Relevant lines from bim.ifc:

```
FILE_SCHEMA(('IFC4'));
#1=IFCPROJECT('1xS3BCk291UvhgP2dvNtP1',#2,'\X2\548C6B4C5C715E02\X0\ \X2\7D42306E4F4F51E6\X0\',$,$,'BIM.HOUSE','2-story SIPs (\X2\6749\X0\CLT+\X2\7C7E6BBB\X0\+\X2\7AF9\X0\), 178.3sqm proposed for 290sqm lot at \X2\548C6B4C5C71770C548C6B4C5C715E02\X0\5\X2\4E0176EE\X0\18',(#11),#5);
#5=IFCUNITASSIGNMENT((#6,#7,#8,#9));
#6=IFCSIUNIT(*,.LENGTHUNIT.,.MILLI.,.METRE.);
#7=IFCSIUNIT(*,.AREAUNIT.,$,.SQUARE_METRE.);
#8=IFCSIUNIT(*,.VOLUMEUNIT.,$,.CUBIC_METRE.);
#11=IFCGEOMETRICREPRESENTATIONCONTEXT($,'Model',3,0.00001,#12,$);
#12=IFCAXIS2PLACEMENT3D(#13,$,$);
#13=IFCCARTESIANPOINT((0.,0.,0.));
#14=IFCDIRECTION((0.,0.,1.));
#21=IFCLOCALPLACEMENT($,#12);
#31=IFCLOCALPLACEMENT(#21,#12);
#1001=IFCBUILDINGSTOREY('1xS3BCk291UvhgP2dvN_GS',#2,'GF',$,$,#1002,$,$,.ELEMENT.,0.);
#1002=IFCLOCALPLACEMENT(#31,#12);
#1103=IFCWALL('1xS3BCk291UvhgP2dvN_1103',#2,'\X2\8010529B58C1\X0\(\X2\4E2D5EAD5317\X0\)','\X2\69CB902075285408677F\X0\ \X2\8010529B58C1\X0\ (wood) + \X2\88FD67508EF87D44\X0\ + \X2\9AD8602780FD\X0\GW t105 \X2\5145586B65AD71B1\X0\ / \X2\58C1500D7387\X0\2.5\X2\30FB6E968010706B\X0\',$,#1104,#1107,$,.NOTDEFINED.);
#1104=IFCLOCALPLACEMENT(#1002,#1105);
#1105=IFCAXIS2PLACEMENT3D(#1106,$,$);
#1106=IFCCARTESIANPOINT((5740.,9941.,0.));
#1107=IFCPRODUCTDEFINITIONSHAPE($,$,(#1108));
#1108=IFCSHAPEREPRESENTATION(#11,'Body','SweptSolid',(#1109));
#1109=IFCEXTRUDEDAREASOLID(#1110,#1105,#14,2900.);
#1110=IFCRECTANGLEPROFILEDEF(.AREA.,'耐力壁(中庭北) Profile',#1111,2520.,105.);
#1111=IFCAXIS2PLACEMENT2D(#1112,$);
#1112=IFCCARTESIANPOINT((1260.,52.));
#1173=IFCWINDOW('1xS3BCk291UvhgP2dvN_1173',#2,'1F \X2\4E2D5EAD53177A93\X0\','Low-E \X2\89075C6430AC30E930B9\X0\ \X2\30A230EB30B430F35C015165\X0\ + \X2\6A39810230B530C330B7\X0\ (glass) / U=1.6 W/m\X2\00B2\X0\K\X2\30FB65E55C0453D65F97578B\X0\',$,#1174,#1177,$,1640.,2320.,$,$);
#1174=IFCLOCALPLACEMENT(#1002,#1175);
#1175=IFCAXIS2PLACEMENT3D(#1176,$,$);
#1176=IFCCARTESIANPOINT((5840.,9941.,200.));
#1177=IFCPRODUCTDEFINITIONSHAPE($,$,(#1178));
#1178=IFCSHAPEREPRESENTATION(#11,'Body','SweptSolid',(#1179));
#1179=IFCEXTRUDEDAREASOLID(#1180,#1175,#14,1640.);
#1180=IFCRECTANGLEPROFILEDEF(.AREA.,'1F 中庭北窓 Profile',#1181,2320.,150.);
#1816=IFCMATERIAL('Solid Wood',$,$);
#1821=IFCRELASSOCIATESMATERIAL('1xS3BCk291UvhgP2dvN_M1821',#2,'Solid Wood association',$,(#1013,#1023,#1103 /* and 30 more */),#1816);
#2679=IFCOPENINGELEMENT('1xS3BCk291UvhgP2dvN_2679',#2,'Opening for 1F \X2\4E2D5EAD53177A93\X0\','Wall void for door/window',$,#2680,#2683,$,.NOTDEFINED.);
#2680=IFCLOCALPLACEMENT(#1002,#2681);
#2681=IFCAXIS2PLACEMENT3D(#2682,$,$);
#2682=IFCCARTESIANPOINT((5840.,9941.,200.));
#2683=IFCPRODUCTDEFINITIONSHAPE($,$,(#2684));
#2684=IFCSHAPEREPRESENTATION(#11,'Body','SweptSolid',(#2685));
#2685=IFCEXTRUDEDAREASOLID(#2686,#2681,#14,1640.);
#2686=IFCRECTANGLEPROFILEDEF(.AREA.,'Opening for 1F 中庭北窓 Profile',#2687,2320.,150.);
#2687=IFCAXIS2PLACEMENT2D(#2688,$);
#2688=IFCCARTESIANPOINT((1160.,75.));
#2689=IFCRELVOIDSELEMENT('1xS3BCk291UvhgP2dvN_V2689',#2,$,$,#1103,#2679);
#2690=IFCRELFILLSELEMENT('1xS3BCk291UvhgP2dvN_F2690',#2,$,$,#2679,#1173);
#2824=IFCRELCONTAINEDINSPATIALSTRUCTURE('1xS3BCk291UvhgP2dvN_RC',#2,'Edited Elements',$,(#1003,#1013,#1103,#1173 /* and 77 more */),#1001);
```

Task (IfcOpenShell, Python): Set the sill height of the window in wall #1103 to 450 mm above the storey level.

```python
import numpy as np
import ifcopenshell
import ifcopenshell.api.geometry
import ifcopenshell.geom
import ifcopenshell.util.element
import ifcopenshell.util.placement
import ifcopenshell.util.shape
import ifcopenshell.util.unit

model = ifcopenshell.open("bim.ifc")
unit_scale = ifcopenshell.util.unit.calculate_unit_scale(model)

window = model.by_guid("1xS3BCk291UvhgP2dvN_1173")
opening = window.FillsVoids[0].RelatingOpeningElement
storey = ifcopenshell.util.element.get_container(window, ifc_class="IfcBuildingStorey")
level = ifcopenshell.util.placement.get_local_placement(storey.ObjectPlacement)[2, 3]

# The opening's origin need not be at the sill, so measure its lowest point.
shape = ifcopenshell.geom.create_shape(ifcopenshell.geom.settings(), opening)
bottom = ifcopenshell.util.shape.get_shape_bottom_elevation(shape, shape.geometry) / unit_scale
dz = level + 450.0 - bottom

shift = np.array([0.0, 0.0, dz])
# The window is not placed relative to its opening, so move both.
for product in (opening, window):
    matrix = ifcopenshell.util.placement.get_local_placement(product.ObjectPlacement)
    matrix[:3, 3] += shift
    ifcopenshell.api.geometry.edit_object_placement(model, product=product, matrix=matrix, is_si=False)

print(f"moved by {dz * unit_scale:+.3f} m")

model.write("bim_v2.ifc")
```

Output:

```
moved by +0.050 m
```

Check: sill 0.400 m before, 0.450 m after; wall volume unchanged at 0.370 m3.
